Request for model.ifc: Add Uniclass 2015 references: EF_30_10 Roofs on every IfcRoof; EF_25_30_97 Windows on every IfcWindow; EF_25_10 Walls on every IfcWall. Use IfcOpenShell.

First a look at what the model holds.

```python
import ifcopenshell

model = ifcopenshell.open("model.ifc")
print(model.schema)
print("classifications:", [c.Name for c in model.by_type("IfcClassification")])
for ifc_class in ("IfcDoor", "IfcRoof", "IfcStair", "IfcWall", "IfcWindow"):
    print(ifc_class, len(model.by_type(ifc_class)))
```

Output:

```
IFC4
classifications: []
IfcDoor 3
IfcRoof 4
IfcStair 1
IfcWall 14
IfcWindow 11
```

```python
import ifcopenshell
import ifcopenshell.api.classification

model = ifcopenshell.open("model.ifc")

system = ifcopenshell.api.classification.add_classification(model, classification="Uniclass 2015")

codes = {
    "IfcRoof": ("EF_30_10", "Roofs"),
    "IfcWindow": ("EF_25_30_97", "Windows"),
    "IfcWall": ("EF_25_10", "Walls"),
}
for ifc_class, (code, name) in codes.items():
    products = model.by_type(ifc_class)
    ifcopenshell.api.classification.add_reference(
        model, products=products, classification=system, identification=code, name=name
    )
    print(code, len(products))

model.write("model_rev.ifc")
```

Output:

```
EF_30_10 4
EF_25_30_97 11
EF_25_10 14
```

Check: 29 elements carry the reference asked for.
